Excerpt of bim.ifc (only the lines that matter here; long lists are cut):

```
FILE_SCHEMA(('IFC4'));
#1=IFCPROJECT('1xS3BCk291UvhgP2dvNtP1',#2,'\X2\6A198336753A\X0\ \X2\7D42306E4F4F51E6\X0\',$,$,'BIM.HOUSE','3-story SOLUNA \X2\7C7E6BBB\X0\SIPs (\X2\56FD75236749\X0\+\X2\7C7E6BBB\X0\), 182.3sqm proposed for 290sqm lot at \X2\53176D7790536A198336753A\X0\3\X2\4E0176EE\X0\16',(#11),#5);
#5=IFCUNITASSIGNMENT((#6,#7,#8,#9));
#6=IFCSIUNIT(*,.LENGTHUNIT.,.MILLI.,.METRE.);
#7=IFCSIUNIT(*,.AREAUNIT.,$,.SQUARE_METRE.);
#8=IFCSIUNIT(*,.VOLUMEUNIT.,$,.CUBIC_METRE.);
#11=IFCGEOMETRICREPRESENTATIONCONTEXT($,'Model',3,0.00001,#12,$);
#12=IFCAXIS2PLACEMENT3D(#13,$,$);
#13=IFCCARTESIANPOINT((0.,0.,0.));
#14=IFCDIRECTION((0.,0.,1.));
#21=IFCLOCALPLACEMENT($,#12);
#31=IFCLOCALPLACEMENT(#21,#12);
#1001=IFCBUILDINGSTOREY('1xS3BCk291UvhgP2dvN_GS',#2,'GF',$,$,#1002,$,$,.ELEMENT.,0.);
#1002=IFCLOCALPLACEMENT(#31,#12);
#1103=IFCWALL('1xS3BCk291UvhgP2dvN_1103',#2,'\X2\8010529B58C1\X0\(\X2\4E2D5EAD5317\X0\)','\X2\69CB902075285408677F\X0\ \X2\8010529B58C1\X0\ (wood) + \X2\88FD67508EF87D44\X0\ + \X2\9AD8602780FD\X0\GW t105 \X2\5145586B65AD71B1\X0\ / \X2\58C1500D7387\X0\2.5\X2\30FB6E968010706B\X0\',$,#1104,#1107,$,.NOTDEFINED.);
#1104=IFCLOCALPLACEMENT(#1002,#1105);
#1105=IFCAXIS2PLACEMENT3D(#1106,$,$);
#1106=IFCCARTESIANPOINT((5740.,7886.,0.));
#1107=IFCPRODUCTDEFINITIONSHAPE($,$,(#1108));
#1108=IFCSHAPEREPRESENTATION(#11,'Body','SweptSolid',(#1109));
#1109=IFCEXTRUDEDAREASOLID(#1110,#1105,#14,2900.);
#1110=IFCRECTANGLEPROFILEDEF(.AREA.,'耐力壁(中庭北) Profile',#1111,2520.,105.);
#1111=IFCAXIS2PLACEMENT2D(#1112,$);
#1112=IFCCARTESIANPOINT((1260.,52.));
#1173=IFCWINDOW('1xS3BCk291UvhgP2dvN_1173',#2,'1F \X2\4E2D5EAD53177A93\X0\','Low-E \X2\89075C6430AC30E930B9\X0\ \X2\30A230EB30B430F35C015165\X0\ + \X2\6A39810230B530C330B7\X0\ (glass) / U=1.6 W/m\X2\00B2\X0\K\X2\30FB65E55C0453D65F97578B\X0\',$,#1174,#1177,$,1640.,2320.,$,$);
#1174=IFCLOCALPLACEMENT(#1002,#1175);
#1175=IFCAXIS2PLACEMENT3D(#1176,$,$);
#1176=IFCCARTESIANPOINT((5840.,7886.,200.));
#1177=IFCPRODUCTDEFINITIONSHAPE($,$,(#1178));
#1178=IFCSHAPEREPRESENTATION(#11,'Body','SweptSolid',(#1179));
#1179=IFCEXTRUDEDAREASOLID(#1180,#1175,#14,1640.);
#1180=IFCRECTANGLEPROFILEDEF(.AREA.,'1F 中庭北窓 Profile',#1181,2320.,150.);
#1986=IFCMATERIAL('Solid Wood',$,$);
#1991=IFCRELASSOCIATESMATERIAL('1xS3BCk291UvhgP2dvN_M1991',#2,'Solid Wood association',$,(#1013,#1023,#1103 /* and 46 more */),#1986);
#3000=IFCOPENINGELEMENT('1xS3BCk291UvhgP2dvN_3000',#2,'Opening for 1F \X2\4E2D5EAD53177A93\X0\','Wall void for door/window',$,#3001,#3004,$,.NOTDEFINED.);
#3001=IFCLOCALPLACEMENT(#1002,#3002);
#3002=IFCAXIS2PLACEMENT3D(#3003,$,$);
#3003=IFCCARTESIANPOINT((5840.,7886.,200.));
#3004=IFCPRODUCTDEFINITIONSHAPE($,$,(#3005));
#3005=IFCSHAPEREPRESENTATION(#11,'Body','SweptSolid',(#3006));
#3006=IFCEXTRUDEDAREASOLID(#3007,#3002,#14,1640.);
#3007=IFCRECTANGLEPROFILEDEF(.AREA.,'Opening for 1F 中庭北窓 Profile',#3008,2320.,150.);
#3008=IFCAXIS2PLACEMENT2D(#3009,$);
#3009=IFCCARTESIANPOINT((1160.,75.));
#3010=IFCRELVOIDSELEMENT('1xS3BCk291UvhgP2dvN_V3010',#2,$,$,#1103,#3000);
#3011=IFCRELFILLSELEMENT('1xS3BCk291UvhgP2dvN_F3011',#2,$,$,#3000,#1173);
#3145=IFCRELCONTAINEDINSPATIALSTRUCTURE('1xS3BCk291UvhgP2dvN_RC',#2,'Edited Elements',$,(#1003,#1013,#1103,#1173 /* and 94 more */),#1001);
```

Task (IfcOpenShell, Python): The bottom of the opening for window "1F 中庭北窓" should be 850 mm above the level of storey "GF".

```python
import numpy as np
import ifcopenshell
import ifcopenshell.api.geometry
import ifcopenshell.geom
import ifcopenshell.util.element
import ifcopenshell.util.placement
import ifcopenshell.util.shape
import ifcopenshell.util.unit

model = ifcopenshell.open("bim.ifc")
unit_scale = ifcopenshell.util.unit.calculate_unit_scale(model)

window = model.by_guid("1xS3BCk291UvhgP2dvN_1173")
opening = window.FillsVoids[0].RelatingOpeningElement
storey = ifcopenshell.util.element.get_container(window, ifc_class="IfcBuildingStorey")
level = ifcopenshell.util.placement.get_local_placement(storey.ObjectPlacement)[2, 3]

# The opening's origin need not be at the sill, so measure its lowest point.
shape = ifcopenshell.geom.create_shape(ifcopenshell.geom.settings(), opening)
bottom = ifcopenshell.util.shape.get_shape_bottom_elevation(shape, shape.geometry) / unit_scale
dz = level + 0.85 / unit_scale - bottom

shift = np.array([0.0, 0.0, dz])
# The window is not placed relative to its opening, so move both.
for product in (opening, window):
    matrix = ifcopenshell.util.placement.get_local_placement(product.ObjectPlacement)
    matrix[:3, 3] += shift
    ifcopenshell.api.geometry.edit_object_placement(model, product=product, matrix=matrix, is_si=False)

print(f"moved by {dz * unit_scale:+.3f} m")

model.write("bim-out.ifc")
```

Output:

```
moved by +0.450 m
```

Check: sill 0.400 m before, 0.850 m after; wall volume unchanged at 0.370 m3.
